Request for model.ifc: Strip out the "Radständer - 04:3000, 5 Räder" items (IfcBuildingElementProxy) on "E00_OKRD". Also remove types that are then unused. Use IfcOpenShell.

First a look at what the model holds.

```python
import ifcopenshell
import ifcopenshell.util.element

model = ifcopenshell.open("model.ifc")
print(model.schema)
storey = next(s for s in model.by_type("IfcBuildingStorey") if s.Name == "E00_OKRD")
proxies = [e for e in ifcopenshell.util.element.get_decomposition(storey) if e.is_a("IfcBuildingElementProxy")]
seen = {}
for e in proxies:
    element_type = ifcopenshell.util.element.get_type(e)
    name = element_type.Name if element_type not in (None, e) else None
    seen[name] = seen.get(name, 0) + 1
for name, count in sorted(seen.items(), key=str):
    print(count, "x", name)
```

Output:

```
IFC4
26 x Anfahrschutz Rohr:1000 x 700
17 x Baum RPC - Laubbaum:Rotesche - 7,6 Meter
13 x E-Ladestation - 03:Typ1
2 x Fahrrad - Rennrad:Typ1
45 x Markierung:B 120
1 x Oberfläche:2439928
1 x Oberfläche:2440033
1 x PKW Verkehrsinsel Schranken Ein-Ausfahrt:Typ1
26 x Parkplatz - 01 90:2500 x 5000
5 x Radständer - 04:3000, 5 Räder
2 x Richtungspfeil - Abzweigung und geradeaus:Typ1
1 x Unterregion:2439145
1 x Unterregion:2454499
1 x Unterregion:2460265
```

```python
import ifcopenshell
import ifcopenshell.api.root
import ifcopenshell.util.element

model = ifcopenshell.open("model.ifc")

storey = next(s for s in model.by_type("IfcBuildingStorey") if s.Name == "E00_OKRD")
proxies = [e for e in ifcopenshell.util.element.get_decomposition(storey) if e.is_a("IfcBuildingElementProxy")]
targets = [e for e in proxies if (t := ifcopenshell.util.element.get_type(e)) not in (None, e) and t.Name == "Radständer - 04:3000, 5 Räder"]
types = {ifcopenshell.util.element.get_type(e) for e in targets} - {None, *targets}

for e in targets:
    ifcopenshell.api.root.remove_product(model, product=e)
print(len(targets), "removed")

unused = [t for t in types if not ifcopenshell.util.element.get_types(t)]
for t in unused:
    ifcopenshell.api.root.remove_product(model, product=t)
print(len(unused), "unused types removed")

model.write("model_updated.ifc")
```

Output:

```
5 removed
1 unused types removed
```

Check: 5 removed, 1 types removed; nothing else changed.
